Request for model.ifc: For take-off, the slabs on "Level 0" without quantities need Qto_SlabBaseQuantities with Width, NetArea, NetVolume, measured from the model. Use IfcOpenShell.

First a look at what the model holds.

```python
import ifcopenshell
import ifcopenshell.util.element
import ifcopenshell.util.unit

model = ifcopenshell.open("model.ifc")
print(model.schema)
for unit_type in ("LENGTHUNIT", "AREAUNIT", "VOLUMEUNIT"):
    print(unit_type, ifcopenshell.util.unit.calculate_unit_scale(model, unit_type))
storey = next(s for s in model.by_type("IfcBuildingStorey") if s.Name == "Level 0")
slabs = [e for e in ifcopenshell.util.element.get_decomposition(storey) if e.is_a("IfcSlab")]
for e in sorted(slabs, key=lambda e: e.id()):
    print(e.id(), e.is_a(), e.Name, list(ifcopenshell.util.element.get_psets(e, qtos_only=True)), sep=" | ")
```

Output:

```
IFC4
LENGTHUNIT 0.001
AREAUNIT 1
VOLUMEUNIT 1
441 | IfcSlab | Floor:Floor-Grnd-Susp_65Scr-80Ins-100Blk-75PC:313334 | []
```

```python
import ifcopenshell
import ifcopenshell.api.pset
import ifcopenshell.geom
import ifcopenshell.util.element
import ifcopenshell.util.shape
import ifcopenshell.util.unit

model = ifcopenshell.open("model.ifc")
unit_scale = ifcopenshell.util.unit.calculate_unit_scale(model)
area_scale = ifcopenshell.util.unit.calculate_unit_scale(model, "AREAUNIT")
volume_scale = ifcopenshell.util.unit.calculate_unit_scale(model, "VOLUMEUNIT")
settings = ifcopenshell.geom.settings()

storey = next(s for s in model.by_type("IfcBuildingStorey") if s.Name == "Level 0")
slabs = [e for e in ifcopenshell.util.element.get_decomposition(storey) if e.is_a("IfcSlab")]

for e in sorted(slabs, key=lambda e: e.id()):
    if ifcopenshell.util.element.get_psets(e, qtos_only=True, should_inherit=False):
        continue
    # Geometry comes back in metres, in the element's own axes.
    shape = ifcopenshell.geom.create_shape(settings, e)
    values = {
        "Width": ifcopenshell.util.shape.get_z(shape.geometry) / unit_scale,
        "NetArea": ifcopenshell.util.shape.get_footprint_area(shape.geometry) / area_scale,
        "NetVolume": ifcopenshell.util.shape.get_volume(shape.geometry) / volume_scale,
    }
    qto = ifcopenshell.api.pset.add_qto(model, product=e, name="Qto_SlabBaseQuantities")
    ifcopenshell.api.pset.edit_qto(model, qto=qto, properties=values)
    print(e.id(), {k: round(v, 3) for k, v in values.items()})

model.write("model_rev.ifc")
```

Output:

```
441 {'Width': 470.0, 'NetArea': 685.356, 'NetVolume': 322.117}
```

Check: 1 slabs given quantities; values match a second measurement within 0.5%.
